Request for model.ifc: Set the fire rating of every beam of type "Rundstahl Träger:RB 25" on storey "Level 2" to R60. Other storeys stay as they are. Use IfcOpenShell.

First a look at what the model holds.

```python
import ifcopenshell
import ifcopenshell.util.element

model = ifcopenshell.open("model.ifc")
print(model.schema)
storey = next(s for s in model.by_type("IfcBuildingStorey") if s.Name == "Level 2")
beams = [e for e in ifcopenshell.util.element.get_decomposition(storey) if e.is_a("IfcBeam")]
seen = {}
for e in beams:
    element_type = ifcopenshell.util.element.get_type(e)
    key = (element_type.Name if element_type != e and element_type else None, ifcopenshell.util.element.get_pset(e, "Pset_BeamCommon", "FireRating"))
    seen[key] = seen.get(key, 0) + 1
for (name, value), count in sorted(seen.items(), key=str):
    print(count, "x", name, "|", value)
```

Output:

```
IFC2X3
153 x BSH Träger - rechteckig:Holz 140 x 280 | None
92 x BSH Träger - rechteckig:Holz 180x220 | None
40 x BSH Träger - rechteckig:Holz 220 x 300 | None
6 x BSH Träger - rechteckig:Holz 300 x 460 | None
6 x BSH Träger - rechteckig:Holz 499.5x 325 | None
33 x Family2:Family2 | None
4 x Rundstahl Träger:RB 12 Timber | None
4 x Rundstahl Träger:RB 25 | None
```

```python
import ifcopenshell
import ifcopenshell.api.pset
import ifcopenshell.util.element

model = ifcopenshell.open("model.ifc")

storey = next(s for s in model.by_type("IfcBuildingStorey") if s.Name == "Level 2")
beams = [e for e in ifcopenshell.util.element.get_decomposition(storey) if e.is_a("IfcBeam")]

count = 0
for e in beams:
    element_type = ifcopenshell.util.element.get_type(e)
    if element_type in (None, e) or element_type.Name != "Rundstahl Träger:RB 25":
        continue
    # add_pset returns the element's existing set when there is one.
    pset = ifcopenshell.api.pset.add_pset(model, product=e, name="Pset_BeamCommon")
    ifcopenshell.api.pset.edit_pset(model, pset=pset, properties={"FireRating": "R60"})
    count += 1

print(count, "beams updated")

model.write("model_v2.ifc")
```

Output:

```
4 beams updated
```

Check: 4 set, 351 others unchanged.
